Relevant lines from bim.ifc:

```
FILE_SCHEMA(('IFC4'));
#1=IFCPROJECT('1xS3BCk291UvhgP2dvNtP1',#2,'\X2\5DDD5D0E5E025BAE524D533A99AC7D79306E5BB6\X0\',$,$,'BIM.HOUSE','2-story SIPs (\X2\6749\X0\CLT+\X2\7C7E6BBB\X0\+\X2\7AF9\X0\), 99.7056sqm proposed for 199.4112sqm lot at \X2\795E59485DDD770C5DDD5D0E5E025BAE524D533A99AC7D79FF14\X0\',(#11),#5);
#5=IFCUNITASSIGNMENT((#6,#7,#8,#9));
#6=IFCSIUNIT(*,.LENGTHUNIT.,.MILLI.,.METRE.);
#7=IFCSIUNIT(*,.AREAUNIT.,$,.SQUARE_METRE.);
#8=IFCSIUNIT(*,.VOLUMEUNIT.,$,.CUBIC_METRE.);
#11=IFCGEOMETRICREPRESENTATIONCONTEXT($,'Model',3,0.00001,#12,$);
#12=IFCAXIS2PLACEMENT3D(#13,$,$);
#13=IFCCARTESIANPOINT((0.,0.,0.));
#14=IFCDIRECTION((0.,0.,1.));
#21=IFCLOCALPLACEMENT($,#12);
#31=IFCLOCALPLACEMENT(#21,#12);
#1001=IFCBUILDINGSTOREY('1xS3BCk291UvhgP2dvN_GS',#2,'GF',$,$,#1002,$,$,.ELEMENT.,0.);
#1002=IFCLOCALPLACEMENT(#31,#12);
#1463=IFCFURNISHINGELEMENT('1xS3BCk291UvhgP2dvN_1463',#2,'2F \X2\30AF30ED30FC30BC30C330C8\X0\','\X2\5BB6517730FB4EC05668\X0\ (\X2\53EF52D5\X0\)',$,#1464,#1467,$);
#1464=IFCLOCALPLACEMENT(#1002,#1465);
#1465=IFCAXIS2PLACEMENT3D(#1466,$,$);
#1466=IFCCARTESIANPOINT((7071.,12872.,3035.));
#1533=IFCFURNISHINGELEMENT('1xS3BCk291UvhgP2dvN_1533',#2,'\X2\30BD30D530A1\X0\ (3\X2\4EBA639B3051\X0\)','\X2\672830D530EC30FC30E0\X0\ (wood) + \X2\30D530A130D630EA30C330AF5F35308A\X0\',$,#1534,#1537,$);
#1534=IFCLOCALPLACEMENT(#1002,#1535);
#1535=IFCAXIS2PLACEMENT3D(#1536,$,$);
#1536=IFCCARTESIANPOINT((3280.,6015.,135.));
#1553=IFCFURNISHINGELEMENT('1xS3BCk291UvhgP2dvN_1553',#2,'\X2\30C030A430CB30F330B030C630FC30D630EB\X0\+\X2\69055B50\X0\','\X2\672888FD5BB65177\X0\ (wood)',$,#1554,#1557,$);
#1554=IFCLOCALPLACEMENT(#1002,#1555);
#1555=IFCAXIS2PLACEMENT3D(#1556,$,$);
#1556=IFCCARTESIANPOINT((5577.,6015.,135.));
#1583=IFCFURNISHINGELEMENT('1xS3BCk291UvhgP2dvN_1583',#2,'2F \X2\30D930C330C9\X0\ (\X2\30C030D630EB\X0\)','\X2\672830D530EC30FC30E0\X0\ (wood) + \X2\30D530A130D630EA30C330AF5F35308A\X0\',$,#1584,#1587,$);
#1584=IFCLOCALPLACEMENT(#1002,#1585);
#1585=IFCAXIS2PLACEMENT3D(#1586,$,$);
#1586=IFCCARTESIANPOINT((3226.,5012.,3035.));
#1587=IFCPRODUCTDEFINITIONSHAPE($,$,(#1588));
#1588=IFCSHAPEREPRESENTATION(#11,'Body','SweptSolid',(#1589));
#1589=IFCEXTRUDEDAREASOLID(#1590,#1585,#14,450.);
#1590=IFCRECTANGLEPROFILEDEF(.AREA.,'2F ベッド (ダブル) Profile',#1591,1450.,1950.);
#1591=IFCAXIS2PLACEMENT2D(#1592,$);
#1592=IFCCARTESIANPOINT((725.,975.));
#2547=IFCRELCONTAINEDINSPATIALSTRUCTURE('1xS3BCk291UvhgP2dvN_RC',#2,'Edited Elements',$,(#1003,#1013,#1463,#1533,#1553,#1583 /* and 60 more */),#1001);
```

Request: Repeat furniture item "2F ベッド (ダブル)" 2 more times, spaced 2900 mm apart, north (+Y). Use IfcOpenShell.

```python
import numpy as np
import ifcopenshell
import ifcopenshell.api.geometry
import ifcopenshell.api.root
import ifcopenshell.util.element
import ifcopenshell.util.placement
import ifcopenshell.util.unit

model = ifcopenshell.open("bim.ifc")
unit_scale = ifcopenshell.util.unit.calculate_unit_scale(model)


def reuse_history(source, copy):
    """copy_class also copies each property set's owner history, people and application; keep the originals."""
    for rel in copy.IsDefinedBy:
        if rel.is_a("IfcRelDefinesByProperties") and (history := rel.RelatingPropertyDefinition.OwnerHistory):
            rel.RelatingPropertyDefinition.OwnerHistory = source.OwnerHistory
            ifcopenshell.util.element.remove_deep2(model, history)


source = model.by_guid("1xS3BCk291UvhgP2dvN_1583")
base = ifcopenshell.util.placement.get_local_placement(source.ObjectPlacement)
step = np.array([0.0, 1.0, 0.0]) * 2.9 / unit_scale

for i in range(1, 3):
    copy = ifcopenshell.api.root.copy_class(model, product=source)
    copy.Representation = ifcopenshell.util.element.copy_deep(
        model, source.Representation, exclude=["IfcGeometricRepresentationContext", "IfcRepresentationMap"]
    )
    reuse_history(source, copy)
    matrix = base.copy()
    matrix[:3, 3] += i * step
    print("added at", matrix[:3, 3].round(3) + 0.0)
    ifcopenshell.api.geometry.edit_object_placement(model, product=copy, matrix=matrix, is_si=False)

model.write("bim_rev.ifc")
```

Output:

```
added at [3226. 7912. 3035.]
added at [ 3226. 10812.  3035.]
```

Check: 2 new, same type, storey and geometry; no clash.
